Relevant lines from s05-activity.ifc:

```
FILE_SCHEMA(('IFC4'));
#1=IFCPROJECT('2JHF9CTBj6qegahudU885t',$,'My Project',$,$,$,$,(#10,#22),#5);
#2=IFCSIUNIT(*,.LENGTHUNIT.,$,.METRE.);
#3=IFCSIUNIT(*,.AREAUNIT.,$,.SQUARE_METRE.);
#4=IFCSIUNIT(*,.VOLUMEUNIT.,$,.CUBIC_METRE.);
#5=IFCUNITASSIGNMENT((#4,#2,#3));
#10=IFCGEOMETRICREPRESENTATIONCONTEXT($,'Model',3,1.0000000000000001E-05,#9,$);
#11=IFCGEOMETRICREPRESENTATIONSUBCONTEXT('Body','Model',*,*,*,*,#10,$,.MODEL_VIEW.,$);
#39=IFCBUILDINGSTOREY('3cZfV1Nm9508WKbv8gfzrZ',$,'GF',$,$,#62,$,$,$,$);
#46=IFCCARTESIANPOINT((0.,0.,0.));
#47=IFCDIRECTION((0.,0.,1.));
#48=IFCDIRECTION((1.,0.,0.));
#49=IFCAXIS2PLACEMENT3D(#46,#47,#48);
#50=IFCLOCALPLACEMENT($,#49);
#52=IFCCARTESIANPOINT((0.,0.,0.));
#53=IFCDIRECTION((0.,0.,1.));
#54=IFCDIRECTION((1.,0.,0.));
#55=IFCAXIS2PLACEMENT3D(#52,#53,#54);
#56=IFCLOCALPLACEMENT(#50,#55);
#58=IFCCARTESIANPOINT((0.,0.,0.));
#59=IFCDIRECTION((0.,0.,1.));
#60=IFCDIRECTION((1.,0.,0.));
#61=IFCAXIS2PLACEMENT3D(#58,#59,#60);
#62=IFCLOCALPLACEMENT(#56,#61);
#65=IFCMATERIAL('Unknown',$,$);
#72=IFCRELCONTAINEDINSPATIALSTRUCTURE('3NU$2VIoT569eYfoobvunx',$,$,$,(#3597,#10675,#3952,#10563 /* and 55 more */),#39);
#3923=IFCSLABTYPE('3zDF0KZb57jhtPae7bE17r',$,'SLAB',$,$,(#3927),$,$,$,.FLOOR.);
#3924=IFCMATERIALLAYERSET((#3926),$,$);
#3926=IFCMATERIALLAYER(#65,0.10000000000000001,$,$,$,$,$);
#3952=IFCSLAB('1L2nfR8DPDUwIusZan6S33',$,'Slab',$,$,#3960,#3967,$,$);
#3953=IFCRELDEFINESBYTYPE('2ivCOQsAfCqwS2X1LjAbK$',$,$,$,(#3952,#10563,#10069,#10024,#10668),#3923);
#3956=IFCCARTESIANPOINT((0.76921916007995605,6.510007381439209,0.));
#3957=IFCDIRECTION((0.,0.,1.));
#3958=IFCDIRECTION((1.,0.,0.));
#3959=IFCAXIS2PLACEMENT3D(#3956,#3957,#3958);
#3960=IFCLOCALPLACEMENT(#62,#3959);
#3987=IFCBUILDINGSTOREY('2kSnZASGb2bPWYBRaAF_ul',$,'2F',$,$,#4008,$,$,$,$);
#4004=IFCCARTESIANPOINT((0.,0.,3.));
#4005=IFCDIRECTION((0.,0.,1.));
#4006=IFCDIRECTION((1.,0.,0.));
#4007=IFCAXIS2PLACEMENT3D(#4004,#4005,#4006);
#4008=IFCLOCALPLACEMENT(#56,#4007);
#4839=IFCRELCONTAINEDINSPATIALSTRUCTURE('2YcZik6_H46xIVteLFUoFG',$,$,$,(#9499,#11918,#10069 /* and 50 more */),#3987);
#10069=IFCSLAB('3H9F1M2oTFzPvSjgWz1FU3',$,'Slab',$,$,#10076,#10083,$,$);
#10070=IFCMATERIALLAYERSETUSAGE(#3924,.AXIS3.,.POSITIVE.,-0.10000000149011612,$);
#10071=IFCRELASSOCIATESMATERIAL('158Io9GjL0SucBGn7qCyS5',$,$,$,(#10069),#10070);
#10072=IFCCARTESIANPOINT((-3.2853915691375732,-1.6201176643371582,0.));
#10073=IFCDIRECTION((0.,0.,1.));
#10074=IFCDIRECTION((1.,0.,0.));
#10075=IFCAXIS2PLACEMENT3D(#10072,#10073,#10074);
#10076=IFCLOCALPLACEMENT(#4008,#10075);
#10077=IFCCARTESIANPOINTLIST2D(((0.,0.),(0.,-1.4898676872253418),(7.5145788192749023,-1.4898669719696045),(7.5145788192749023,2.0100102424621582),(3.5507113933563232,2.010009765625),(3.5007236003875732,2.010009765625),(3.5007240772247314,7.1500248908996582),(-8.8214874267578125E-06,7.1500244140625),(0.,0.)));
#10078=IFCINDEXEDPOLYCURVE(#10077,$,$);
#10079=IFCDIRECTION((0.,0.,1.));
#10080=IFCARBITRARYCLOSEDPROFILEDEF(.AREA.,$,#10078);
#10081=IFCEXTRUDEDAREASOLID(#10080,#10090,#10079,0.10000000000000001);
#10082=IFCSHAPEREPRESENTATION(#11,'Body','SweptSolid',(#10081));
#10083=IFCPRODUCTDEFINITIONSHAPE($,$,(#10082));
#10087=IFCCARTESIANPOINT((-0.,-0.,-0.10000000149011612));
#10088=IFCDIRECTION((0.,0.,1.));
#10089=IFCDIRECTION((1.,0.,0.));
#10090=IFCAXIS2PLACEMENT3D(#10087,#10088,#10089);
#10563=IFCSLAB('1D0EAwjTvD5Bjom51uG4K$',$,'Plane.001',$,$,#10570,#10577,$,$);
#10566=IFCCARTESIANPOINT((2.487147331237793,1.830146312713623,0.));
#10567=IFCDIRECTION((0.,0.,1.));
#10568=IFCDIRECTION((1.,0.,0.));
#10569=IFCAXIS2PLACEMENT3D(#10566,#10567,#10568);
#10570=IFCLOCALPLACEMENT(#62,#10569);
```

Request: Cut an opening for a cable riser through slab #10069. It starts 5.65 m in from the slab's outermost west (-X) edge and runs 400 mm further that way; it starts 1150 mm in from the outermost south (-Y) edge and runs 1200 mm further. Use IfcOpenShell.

```python
import numpy as np
import ifcopenshell
import ifcopenshell.api.feature
import ifcopenshell.api.geometry
import ifcopenshell.api.root
import ifcopenshell.geom
import ifcopenshell.util.placement
import ifcopenshell.util.representation
import ifcopenshell.util.shape
import ifcopenshell.util.unit

model = ifcopenshell.open("s05-activity.ifc")
unit_scale = ifcopenshell.util.unit.calculate_unit_scale(model)
settings = ifcopenshell.geom.settings()


def volume(element):
    """Net volume in cubic metres, openings subtracted."""
    shape = ifcopenshell.geom.create_shape(settings, element)
    return ifcopenshell.util.shape.get_volume(shape.geometry)


slab = model.by_guid("3H9F1M2oTFzPvSjgWz1FU3")
before = volume(slab)

# Extent in the slab's own axes, in metres. The edges named are its -X and -Y sides.
slab_shape = ifcopenshell.geom.create_shape(settings, slab)
vertices = ifcopenshell.util.shape.get_vertices(slab_shape.geometry)
x_min, y_min, bottom = vertices.min(axis=0)
top = vertices[:, 2].max()

opening = ifcopenshell.api.root.create_entity(model, ifc_class="IfcOpeningElement", name="Cable riser opening", predefined_type="OPENING")
context = ifcopenshell.util.representation.get_context(model, "Model", "Body", "MODEL_VIEW")
width, depth = 0.4, 1.2
outline = [(0.0, 0.0), (width, 0.0), (width, depth), (0.0, depth), (0.0, 0.0)]
# Overshoot both faces by 50 mm so the cut is clean.
shape = ifcopenshell.api.geometry.add_slab_representation(
    model, context=context, depth=top - bottom + 0.1, polyline=outline
)
ifcopenshell.api.geometry.assign_representation(model, product=opening, representation=shape)

matrix = ifcopenshell.util.placement.get_local_placement(slab.ObjectPlacement)
matrix[:, 3] = matrix @ np.append(np.array([x_min + 5.65, y_min + 1.15, bottom - 0.05]) / unit_scale, 1.0)
ifcopenshell.api.geometry.edit_object_placement(model, product=opening, matrix=matrix, is_si=False)
ifcopenshell.api.feature.add_feature(model, feature=opening, element=slab)

after = volume(slab)

print(f"slab volume {before:.3f} -> {after:.3f} m3")

model.write("s05-activity-out.ifc")
```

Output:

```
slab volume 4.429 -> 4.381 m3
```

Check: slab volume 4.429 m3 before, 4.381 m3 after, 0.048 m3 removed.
